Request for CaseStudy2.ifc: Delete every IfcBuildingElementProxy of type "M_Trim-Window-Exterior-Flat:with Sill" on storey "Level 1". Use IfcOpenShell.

First a look at what the model holds.

```python
import ifcopenshell
import ifcopenshell.util.element

model = ifcopenshell.open("CaseStudy2.ifc")
print(model.schema)
storey = next(s for s in model.by_type("IfcBuildingStorey") if s.Name == "Level 1")
proxies = [e for e in ifcopenshell.util.element.get_decomposition(storey) if e.is_a("IfcBuildingElementProxy")]
seen = {}
for e in proxies:
    element_type = ifcopenshell.util.element.get_type(e)
    name = element_type.Name if element_type not in (None, e) else None
    seen[name] = seen.get(name, 0) + 1
for name, count in sorted(seen.items(), key=str):
    print(count, "x", name)
```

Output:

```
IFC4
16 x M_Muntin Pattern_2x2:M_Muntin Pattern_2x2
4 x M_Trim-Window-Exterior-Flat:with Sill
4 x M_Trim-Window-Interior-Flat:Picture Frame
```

```python
import ifcopenshell
import ifcopenshell.api.root
import ifcopenshell.util.element

model = ifcopenshell.open("CaseStudy2.ifc")

storey = next(s for s in model.by_type("IfcBuildingStorey") if s.Name == "Level 1")
proxies = [e for e in ifcopenshell.util.element.get_decomposition(storey) if e.is_a("IfcBuildingElementProxy")]
targets = [e for e in proxies if (t := ifcopenshell.util.element.get_type(e)) not in (None, e) and t.Name == "M_Trim-Window-Exterior-Flat:with Sill"]

for e in targets:
    ifcopenshell.api.root.remove_product(model, product=e)
print(len(targets), "removed")

model.write("CaseStudy2_rev.ifc")
```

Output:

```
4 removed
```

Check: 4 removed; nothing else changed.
